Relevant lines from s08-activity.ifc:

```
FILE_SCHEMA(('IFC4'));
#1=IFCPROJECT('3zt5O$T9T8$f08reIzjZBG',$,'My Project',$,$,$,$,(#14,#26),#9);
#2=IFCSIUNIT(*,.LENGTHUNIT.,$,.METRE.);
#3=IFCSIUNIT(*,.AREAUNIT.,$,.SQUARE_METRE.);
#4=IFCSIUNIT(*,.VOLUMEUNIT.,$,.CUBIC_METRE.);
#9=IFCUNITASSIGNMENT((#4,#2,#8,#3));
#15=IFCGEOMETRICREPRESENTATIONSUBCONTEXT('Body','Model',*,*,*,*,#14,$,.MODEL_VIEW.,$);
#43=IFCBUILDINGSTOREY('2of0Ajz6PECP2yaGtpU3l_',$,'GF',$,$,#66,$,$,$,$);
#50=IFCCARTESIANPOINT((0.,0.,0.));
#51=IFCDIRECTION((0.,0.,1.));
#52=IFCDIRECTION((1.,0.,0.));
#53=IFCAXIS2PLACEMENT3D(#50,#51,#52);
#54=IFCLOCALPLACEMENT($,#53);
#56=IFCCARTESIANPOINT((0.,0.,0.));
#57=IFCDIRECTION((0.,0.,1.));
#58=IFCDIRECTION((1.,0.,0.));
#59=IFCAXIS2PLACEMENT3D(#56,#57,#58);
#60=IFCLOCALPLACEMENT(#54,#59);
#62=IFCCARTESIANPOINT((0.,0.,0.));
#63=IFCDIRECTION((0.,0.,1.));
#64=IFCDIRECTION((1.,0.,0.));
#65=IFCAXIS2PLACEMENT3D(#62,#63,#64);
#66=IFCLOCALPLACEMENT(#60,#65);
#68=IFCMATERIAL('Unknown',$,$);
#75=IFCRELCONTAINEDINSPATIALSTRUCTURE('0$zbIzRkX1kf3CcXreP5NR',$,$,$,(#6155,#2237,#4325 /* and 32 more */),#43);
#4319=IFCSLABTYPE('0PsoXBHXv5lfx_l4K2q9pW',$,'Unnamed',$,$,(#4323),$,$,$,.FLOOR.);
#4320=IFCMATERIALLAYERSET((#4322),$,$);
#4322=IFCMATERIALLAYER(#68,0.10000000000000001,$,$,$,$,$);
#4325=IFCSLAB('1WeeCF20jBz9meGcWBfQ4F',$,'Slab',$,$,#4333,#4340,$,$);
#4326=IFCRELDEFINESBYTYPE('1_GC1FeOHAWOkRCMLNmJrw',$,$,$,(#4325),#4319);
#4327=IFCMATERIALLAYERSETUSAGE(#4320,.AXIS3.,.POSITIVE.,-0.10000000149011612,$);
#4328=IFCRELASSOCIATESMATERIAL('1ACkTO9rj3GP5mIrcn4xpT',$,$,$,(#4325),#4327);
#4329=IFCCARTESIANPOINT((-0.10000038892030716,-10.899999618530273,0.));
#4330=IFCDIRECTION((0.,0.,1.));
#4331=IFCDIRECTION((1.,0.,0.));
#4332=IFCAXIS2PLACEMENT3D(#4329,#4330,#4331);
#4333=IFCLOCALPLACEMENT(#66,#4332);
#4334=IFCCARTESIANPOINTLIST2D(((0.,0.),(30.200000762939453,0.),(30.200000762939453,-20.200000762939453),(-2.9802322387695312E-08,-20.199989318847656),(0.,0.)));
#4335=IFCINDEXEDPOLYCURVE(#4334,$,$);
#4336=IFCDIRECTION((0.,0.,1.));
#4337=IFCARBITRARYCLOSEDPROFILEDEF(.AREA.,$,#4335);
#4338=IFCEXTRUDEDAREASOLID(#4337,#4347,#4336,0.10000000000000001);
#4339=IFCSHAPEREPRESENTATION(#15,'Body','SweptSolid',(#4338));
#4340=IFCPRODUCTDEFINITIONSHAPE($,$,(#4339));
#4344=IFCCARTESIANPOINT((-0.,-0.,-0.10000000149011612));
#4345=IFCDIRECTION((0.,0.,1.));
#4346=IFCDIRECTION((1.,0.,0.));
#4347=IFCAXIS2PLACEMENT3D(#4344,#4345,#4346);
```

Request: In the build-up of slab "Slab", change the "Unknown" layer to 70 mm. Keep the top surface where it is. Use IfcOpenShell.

```python
import ifcopenshell
import ifcopenshell.util.element
import ifcopenshell.util.representation
import ifcopenshell.util.unit

model = ifcopenshell.open("s08-activity.ifc")
unit_scale = ifcopenshell.util.unit.calculate_unit_scale(model)

layer_set = model.by_id(4320)
layer = next(l for l in layer_set.MaterialLayers if l.Material and l.Material.Name == "Unknown")
change = 0.07 / unit_scale - layer.LayerThickness
layer.LayerThickness += change

# Geometry does not follow the layer set by itself.
slabs = [e for e in ifcopenshell.util.element.get_elements_by_material(model, layer_set) if e.is_a("IfcSlab")]
for slab in sorted(slabs, key=lambda e: e.id()):
    body = ifcopenshell.util.representation.get_representation(slab, "Model", "Body")
    solid = body.Items[0]
    old_depth = solid.Depth
    solid.Depth += change
    # Extruded upwards: lower the start of the extrusion so the top stays.
    x, y, z = solid.Position.Location.Coordinates
    solid.Position.Location = model.createIfcCartesianPoint((x, y, z - change))
    print(slab.id(), f"{old_depth:g} -> {solid.Depth:g}")

# The layers are counted up from the underside, which has moved.
for usage in {ifcopenshell.util.element.get_material(slab) for slab in slabs}:
    usage.OffsetFromReferenceLine -= change

model.write("s08-activity_v2.ifc")
```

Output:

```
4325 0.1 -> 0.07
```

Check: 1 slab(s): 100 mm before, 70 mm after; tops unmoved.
